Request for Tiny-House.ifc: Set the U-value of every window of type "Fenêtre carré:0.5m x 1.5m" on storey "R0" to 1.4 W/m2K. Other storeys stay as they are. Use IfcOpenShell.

First a look at what the model holds.

```python
import ifcopenshell
import ifcopenshell.util.element

model = ifcopenshell.open("Tiny-House.ifc")
print(model.schema)
storey = next(s for s in model.by_type("IfcBuildingStorey") if s.Name == "R0")
windows = [e for e in ifcopenshell.util.element.get_decomposition(storey) if e.is_a("IfcWindow")]
seen = {}
for e in windows:
    element_type = ifcopenshell.util.element.get_type(e)
    key = (element_type.Name if element_type != e and element_type else None, ifcopenshell.util.element.get_pset(e, "Pset_WindowCommon", "ThermalTransmittance"))
    seen[key] = seen.get(key, 0) + 1
for (name, value), count in sorted(seen.items(), key=str):
    print(count, "x", name, "|", value)
```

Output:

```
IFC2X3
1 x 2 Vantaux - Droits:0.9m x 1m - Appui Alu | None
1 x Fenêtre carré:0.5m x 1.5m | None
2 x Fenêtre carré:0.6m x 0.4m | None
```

```python
import ifcopenshell
import ifcopenshell.api.pset
import ifcopenshell.util.element

model = ifcopenshell.open("Tiny-House.ifc")

storey = next(s for s in model.by_type("IfcBuildingStorey") if s.Name == "R0")
windows = [e for e in ifcopenshell.util.element.get_decomposition(storey) if e.is_a("IfcWindow")]

count = 0
for e in windows:
    element_type = ifcopenshell.util.element.get_type(e)
    if element_type in (None, e) or element_type.Name != "Fenêtre carré:0.5m x 1.5m":
        continue
    # add_pset returns the element's existing set when there is one.
    pset = ifcopenshell.api.pset.add_pset(model, product=e, name="Pset_WindowCommon")
    ifcopenshell.api.pset.edit_pset(model, pset=pset, properties={"ThermalTransmittance": 1.4})
    count += 1

print(count, "windows updated")

model.write("Tiny-House_updated.ifc")
```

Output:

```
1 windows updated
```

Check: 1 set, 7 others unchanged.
